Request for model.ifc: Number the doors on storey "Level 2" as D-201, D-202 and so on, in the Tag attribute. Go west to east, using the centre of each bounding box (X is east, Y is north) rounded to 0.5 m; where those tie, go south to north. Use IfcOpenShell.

First a look at what the model holds.

```python
import ifcopenshell
import ifcopenshell.util.element
import ifcopenshell.util.placement

model = ifcopenshell.open("model.ifc")
print(model.schema)
storey = next(s for s in model.by_type("IfcBuildingStorey") if s.Name == "Level 2")
doors = [e for e in ifcopenshell.util.element.get_decomposition(storey) if e.is_a("IfcDoor")]
for e in sorted(doors, key=lambda e: e.id()):
    origin = ifcopenshell.util.placement.get_local_placement(e.ObjectPlacement)[:3, 3]
    print(e.id(), e.Tag, e.Name, origin.round(2) + 0.0, sep=" | ")
```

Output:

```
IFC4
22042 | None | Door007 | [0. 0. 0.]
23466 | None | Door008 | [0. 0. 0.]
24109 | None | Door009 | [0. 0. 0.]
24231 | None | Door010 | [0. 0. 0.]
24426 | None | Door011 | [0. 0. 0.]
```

```python
import ifcopenshell
import ifcopenshell.geom
import ifcopenshell.util.element
import ifcopenshell.util.shape

model = ifcopenshell.open("model.ifc")
settings = ifcopenshell.geom.settings()
settings.set("use-world-coords", True)


def centre(element):
    shape = ifcopenshell.geom.create_shape(settings, element)
    return ifcopenshell.util.shape.get_bbox_centroid(shape.geometry)


storey = next(s for s in model.by_type("IfcBuildingStorey") if s.Name == "Level 2")
doors = [e for e in ifcopenshell.util.element.get_decomposition(storey) if e.is_a("IfcDoor")]

# Insertion points can sit at a corner or the storey origin, so sort by the geometry (in metres).
centres = {e: centre(e) for e in doors}
doors.sort(key=lambda e: (round(centres[e][0] / 0.5), centres[e][1]))

for i, e in enumerate(doors, start=1):
    number = f"D-2{i:02d}"
    e.Tag = number
    print(e.id(), number)

model.write("model_edited.ifc")
```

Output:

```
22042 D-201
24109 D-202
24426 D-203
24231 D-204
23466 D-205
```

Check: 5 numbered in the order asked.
